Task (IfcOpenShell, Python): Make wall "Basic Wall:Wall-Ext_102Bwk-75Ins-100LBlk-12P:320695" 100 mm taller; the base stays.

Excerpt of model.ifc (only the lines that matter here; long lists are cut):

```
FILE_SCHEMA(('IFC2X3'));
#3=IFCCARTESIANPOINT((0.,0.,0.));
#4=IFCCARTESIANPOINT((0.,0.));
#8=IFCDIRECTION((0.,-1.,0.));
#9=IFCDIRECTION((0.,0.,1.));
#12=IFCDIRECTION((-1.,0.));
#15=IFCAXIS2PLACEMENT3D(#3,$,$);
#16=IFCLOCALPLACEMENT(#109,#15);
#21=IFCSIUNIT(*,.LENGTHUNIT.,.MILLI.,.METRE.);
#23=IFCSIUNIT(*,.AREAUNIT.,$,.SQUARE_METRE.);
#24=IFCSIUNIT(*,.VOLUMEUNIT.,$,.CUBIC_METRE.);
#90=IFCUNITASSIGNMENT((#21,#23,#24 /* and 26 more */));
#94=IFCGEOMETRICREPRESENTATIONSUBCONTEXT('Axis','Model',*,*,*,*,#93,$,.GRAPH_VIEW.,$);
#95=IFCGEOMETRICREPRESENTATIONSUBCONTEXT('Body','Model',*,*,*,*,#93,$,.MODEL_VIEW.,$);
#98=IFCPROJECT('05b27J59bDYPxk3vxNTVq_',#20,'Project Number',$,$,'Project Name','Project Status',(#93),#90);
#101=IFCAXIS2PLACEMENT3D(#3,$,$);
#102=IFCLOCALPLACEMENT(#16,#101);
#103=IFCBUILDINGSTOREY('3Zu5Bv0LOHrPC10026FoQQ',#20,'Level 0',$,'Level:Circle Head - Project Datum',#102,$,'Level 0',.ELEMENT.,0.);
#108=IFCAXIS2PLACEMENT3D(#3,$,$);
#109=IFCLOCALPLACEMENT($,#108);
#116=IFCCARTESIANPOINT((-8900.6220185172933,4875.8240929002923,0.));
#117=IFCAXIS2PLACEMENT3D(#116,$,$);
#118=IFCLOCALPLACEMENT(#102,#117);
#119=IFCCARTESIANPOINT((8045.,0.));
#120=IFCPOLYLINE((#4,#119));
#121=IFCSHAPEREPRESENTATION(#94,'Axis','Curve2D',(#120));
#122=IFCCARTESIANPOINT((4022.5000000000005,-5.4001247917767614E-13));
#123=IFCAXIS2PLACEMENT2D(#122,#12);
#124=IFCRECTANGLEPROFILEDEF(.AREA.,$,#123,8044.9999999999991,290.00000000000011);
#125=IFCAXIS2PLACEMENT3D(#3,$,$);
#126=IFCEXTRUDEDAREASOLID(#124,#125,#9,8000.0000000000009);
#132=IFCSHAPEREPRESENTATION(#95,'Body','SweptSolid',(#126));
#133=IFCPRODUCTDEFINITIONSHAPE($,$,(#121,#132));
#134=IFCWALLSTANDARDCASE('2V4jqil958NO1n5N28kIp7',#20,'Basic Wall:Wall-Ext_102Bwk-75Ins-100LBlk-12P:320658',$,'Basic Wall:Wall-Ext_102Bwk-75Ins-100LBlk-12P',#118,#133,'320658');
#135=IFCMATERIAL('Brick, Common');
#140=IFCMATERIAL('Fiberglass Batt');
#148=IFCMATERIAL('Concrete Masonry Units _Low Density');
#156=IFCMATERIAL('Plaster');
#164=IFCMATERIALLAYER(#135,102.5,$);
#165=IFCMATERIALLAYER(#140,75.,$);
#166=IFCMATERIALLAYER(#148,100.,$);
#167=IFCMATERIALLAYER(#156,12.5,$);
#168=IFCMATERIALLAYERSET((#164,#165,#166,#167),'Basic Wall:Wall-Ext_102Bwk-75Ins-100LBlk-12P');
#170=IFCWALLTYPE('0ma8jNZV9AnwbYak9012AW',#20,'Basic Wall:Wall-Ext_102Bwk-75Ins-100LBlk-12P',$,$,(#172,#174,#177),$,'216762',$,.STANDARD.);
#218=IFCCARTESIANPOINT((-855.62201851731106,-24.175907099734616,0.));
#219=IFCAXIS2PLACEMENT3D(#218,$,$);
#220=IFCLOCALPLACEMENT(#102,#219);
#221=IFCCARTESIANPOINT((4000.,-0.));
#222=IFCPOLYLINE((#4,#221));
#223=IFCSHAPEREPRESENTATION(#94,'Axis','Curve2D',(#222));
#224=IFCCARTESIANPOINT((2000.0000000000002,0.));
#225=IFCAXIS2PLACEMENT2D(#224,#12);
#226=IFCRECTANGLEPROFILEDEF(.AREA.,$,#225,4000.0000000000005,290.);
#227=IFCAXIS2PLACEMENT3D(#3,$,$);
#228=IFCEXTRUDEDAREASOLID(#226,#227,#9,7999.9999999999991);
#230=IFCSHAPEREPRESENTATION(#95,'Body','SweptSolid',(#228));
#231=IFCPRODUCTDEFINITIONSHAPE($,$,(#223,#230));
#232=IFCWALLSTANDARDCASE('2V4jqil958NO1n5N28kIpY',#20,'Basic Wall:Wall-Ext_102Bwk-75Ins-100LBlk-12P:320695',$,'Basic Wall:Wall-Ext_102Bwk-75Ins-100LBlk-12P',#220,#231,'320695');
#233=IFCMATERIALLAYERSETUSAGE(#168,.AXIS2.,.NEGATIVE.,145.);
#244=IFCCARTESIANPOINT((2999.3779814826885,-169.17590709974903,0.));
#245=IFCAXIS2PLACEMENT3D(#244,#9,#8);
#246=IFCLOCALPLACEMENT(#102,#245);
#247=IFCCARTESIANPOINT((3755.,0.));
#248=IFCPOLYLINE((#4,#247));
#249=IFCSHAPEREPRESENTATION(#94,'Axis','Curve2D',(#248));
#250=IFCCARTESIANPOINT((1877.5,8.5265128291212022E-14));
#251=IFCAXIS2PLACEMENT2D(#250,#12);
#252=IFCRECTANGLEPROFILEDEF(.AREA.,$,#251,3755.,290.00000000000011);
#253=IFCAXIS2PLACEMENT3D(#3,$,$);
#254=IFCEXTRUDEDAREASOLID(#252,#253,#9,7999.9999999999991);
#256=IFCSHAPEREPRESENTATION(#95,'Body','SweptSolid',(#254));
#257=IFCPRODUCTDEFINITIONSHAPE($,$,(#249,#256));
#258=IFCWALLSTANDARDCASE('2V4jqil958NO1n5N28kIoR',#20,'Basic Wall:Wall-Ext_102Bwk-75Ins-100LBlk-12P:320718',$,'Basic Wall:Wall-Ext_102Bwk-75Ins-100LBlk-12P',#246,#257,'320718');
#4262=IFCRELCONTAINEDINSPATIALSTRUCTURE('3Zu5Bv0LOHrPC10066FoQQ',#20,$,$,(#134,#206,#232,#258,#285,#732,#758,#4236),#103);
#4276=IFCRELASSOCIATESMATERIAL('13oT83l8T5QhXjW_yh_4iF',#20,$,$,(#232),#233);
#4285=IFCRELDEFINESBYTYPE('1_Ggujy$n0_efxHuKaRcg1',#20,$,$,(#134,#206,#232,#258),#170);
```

```python
import ifcopenshell
import ifcopenshell.geom
import ifcopenshell.util.representation
import ifcopenshell.util.shape

model = ifcopenshell.open("model.ifc")
settings = ifcopenshell.geom.settings()


def volume(element):
    """Net volume in cubic metres, openings subtracted."""
    shape = ifcopenshell.geom.create_shape(settings, element)
    return ifcopenshell.util.shape.get_volume(shape.geometry)


wall = model.by_guid("2V4jqil958NO1n5N28kIpY")
before = volume(wall)

body = ifcopenshell.util.representation.get_representation(wall, "Model", "Body")
solid = body.Items[0]
old_height = solid.Depth
solid.Depth += 100.0
after = volume(wall)

print(f"height {old_height:g} -> {solid.Depth:g}, volume {before:.3f} -> {after:.3f} m3")

model.write("model_updated.ifc")
```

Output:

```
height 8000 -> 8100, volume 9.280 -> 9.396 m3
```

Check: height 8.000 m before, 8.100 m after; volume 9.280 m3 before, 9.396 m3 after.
